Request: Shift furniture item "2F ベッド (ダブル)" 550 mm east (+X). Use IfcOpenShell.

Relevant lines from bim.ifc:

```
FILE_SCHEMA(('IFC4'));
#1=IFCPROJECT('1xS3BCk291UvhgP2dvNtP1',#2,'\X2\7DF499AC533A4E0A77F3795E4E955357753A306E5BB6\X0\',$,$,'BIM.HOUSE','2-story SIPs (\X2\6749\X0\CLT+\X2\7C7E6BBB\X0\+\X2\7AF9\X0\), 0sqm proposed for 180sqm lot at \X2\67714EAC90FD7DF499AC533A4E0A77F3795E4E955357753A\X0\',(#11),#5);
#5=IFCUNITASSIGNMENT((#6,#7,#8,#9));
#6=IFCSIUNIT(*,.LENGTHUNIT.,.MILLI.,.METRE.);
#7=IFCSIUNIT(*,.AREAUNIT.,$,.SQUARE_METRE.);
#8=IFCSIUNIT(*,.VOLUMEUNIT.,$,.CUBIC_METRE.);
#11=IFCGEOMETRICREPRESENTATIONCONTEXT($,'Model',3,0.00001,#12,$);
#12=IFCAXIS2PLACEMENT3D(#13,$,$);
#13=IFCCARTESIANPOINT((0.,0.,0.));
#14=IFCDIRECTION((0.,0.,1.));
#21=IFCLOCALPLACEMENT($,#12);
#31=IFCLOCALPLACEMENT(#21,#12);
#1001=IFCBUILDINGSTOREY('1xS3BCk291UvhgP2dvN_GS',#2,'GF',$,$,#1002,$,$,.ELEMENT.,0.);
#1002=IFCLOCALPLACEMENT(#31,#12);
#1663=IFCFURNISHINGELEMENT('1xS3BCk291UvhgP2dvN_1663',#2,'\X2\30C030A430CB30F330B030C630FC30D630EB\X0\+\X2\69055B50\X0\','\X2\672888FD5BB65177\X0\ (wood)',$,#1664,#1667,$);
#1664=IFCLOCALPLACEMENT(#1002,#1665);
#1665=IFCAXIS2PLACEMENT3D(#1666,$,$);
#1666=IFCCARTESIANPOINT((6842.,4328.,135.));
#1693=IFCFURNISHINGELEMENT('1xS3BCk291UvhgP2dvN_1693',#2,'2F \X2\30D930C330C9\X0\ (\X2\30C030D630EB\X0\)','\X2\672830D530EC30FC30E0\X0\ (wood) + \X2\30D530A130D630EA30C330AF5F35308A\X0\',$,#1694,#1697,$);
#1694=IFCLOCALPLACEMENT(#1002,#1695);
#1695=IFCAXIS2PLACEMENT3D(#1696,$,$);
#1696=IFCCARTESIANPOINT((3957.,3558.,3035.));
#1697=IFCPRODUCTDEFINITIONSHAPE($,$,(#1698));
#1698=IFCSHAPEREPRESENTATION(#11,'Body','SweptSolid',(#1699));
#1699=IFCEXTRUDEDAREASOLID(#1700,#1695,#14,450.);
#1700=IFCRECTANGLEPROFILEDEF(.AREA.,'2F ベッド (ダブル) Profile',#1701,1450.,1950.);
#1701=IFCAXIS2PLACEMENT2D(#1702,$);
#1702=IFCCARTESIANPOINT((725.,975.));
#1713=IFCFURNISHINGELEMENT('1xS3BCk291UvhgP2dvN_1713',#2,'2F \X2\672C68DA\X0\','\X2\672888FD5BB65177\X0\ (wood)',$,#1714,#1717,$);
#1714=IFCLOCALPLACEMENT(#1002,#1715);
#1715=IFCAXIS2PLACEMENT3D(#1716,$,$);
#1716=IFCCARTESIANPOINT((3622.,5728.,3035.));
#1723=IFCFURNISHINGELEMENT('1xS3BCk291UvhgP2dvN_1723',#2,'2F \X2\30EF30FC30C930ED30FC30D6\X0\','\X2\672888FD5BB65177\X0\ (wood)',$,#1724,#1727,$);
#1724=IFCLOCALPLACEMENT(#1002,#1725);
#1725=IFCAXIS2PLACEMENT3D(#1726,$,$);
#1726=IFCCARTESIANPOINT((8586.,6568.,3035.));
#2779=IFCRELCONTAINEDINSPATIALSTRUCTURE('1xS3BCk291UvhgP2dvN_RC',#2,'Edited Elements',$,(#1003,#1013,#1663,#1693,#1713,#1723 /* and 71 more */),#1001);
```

```python
import ifcopenshell
import ifcopenshell.api.geometry
import ifcopenshell.util.placement
import ifcopenshell.util.unit

model = ifcopenshell.open("bim.ifc")
unit_scale = ifcopenshell.util.unit.calculate_unit_scale(model)

item = model.by_id(1693)
matrix = ifcopenshell.util.placement.get_local_placement(item.ObjectPlacement)
matrix[0, 3] += 0.55 / unit_scale
ifcopenshell.api.geometry.edit_object_placement(model, product=item, matrix=matrix, is_si=False)

print(ifcopenshell.util.placement.get_local_placement(item.ObjectPlacement).round(3) + 0.0)

model.write("bim-out.ifc")
```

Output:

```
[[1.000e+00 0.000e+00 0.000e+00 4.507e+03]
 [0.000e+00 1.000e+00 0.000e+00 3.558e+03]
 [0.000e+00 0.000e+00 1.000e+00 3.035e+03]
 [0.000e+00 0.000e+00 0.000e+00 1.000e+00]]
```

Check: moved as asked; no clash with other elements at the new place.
